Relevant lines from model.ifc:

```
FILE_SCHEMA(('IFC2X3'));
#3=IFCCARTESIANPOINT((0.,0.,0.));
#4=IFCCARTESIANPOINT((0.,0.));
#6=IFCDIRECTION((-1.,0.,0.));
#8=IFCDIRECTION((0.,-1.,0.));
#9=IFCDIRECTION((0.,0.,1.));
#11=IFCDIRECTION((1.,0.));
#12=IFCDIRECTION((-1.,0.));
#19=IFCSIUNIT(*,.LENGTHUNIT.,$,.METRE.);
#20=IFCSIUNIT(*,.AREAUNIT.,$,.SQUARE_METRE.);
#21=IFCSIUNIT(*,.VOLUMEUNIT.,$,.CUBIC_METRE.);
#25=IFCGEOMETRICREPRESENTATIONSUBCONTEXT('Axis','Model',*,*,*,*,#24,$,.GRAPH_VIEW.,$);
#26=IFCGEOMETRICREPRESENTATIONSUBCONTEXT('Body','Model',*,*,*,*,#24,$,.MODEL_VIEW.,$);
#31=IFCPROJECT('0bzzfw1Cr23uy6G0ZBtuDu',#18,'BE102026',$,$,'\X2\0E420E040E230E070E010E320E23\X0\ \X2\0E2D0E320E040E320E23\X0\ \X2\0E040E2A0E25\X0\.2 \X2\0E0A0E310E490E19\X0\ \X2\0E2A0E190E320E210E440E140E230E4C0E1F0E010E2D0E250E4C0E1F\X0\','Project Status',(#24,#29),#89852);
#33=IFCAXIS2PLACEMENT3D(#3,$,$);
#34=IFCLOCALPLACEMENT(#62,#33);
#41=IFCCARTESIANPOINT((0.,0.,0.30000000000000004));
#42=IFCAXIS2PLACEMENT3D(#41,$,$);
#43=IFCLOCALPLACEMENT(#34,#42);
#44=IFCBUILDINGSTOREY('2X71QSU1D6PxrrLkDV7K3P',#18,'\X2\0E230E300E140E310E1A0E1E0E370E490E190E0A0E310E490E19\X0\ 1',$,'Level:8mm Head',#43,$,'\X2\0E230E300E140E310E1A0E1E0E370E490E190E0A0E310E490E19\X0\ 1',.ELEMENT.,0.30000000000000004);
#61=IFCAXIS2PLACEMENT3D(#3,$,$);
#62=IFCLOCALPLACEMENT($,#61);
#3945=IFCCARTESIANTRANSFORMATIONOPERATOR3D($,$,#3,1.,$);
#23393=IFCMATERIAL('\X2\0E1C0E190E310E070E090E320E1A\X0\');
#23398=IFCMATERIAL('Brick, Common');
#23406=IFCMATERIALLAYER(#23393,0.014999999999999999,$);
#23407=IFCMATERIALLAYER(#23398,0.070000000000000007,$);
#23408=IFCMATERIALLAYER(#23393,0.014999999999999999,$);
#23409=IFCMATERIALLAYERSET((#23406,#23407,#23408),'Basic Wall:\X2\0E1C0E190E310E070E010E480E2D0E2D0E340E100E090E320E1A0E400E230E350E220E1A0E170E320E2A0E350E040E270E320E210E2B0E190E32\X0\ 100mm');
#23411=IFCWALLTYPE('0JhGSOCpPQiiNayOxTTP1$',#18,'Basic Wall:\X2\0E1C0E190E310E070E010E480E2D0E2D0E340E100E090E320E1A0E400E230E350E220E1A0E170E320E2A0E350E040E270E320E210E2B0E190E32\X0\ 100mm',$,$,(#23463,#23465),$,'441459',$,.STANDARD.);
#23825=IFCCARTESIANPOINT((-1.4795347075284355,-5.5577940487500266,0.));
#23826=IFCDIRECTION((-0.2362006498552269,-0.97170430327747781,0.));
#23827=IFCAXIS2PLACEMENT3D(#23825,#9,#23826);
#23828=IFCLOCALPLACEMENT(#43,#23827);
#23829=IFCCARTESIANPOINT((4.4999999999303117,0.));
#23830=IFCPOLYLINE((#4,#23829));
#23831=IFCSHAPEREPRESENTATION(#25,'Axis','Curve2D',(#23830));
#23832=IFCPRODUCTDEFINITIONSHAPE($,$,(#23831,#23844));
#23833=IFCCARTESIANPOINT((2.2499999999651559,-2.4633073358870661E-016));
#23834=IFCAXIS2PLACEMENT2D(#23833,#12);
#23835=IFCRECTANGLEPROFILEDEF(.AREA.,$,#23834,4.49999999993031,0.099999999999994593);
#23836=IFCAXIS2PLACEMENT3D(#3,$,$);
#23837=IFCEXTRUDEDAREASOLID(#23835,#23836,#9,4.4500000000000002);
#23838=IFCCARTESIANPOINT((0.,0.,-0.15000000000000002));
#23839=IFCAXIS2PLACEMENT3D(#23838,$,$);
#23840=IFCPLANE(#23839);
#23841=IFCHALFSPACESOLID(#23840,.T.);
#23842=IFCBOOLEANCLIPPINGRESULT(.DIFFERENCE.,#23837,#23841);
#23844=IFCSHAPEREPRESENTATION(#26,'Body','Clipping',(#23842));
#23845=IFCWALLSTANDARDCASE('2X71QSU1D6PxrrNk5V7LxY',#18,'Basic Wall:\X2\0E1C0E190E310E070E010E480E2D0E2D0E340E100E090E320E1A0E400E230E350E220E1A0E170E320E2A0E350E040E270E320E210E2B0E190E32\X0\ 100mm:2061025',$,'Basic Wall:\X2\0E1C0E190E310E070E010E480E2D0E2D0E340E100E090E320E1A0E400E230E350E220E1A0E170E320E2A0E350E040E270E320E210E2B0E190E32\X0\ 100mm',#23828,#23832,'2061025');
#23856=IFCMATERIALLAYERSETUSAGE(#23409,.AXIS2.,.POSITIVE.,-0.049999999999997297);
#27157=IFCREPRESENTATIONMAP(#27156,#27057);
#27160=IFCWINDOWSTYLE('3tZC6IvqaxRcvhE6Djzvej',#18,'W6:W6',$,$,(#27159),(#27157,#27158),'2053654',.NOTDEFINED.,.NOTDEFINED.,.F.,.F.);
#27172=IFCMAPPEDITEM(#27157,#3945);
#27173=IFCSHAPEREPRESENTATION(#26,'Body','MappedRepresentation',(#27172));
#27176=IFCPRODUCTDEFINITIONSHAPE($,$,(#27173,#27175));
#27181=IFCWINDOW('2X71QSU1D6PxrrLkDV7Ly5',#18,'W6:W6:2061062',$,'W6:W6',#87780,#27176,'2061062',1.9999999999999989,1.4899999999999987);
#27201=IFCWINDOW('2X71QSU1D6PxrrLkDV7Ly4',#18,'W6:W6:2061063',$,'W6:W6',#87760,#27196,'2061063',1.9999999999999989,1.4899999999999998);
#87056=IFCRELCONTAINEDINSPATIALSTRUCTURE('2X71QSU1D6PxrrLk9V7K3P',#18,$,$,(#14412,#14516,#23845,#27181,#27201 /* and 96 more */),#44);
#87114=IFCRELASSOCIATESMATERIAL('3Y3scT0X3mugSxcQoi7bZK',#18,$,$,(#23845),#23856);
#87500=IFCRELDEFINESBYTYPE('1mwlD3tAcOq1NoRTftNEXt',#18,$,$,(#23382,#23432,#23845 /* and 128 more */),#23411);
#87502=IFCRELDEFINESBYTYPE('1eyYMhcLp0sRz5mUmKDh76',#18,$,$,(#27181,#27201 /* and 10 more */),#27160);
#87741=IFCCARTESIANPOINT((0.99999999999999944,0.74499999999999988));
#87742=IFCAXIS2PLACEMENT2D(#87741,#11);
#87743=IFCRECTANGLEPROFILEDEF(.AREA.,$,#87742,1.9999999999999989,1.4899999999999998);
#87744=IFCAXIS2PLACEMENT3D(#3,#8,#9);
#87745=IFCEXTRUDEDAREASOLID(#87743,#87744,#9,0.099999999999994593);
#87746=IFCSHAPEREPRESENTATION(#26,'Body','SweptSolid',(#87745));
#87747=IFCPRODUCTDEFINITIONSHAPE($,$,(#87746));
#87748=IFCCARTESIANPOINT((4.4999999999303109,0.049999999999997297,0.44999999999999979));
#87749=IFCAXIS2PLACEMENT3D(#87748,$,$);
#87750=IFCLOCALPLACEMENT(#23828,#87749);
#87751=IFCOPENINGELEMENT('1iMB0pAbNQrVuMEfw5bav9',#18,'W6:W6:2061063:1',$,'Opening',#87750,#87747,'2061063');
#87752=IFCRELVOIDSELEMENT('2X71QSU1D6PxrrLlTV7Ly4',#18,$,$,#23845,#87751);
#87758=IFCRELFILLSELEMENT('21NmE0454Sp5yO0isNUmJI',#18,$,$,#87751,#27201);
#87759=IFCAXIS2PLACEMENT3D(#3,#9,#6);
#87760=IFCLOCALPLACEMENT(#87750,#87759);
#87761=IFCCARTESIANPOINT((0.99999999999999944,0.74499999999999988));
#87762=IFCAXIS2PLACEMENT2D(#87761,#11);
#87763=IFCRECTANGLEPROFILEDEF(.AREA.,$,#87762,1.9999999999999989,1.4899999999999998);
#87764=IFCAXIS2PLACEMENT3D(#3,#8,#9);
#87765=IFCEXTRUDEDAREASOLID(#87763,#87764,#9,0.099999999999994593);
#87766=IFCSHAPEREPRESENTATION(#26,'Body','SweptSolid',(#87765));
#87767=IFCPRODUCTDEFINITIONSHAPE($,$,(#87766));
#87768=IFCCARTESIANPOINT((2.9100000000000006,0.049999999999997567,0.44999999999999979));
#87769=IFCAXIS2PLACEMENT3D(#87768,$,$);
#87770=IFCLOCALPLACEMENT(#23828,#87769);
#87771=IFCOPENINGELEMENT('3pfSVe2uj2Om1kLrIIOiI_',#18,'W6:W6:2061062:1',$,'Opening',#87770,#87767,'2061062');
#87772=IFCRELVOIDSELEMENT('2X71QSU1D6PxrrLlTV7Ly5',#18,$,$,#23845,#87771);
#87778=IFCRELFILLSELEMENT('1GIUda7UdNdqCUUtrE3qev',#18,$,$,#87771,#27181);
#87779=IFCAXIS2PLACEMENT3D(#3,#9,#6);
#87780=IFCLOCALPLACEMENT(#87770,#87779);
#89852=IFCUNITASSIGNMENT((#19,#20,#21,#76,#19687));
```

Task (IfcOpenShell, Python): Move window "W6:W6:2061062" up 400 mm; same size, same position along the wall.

```python
import numpy as np
import ifcopenshell
import ifcopenshell.api.geometry
import ifcopenshell.util.placement
import ifcopenshell.util.unit

model = ifcopenshell.open("model.ifc")
unit_scale = ifcopenshell.util.unit.calculate_unit_scale(model)

window = model.by_guid("2X71QSU1D6PxrrLkDV7Ly5")
opening = window.FillsVoids[0].RelatingOpeningElement
dz = 0.4 / unit_scale

shift = np.array([0.0, 0.0, dz])
# The window is placed relative to its opening, so it follows when the opening moves.
matrix = ifcopenshell.util.placement.get_local_placement(opening.ObjectPlacement)
matrix[:3, 3] += shift
ifcopenshell.api.geometry.edit_object_placement(
    model, product=opening, matrix=matrix, is_si=False, should_transform_children=True
)

print(f"moved by {dz * unit_scale:+.3f} m")

model.write("model_edited.ifc")
```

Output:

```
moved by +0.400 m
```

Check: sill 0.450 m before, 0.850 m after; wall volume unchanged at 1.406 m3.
